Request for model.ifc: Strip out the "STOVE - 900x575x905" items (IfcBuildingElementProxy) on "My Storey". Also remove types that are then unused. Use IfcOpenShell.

First a look at what the model holds.

```python
import ifcopenshell
import ifcopenshell.util.element

model = ifcopenshell.open("model.ifc")
print(model.schema)
storey = next(s for s in model.by_type("IfcBuildingStorey") if s.Name == "My Storey")
proxies = [e for e in ifcopenshell.util.element.get_decomposition(storey) if e.is_a("IfcBuildingElementProxy")]
seen = {}
for e in proxies:
    element_type = ifcopenshell.util.element.get_type(e)
    name = element_type.Name if element_type not in (None, e) else None
    seen[name] = seen.get(name, 0) + 1
for name, count in sorted(seen.items(), key=str):
    print(count, "x", name)
```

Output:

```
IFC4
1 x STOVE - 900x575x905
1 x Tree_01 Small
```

```python
import ifcopenshell
import ifcopenshell.api.root
import ifcopenshell.util.element

model = ifcopenshell.open("model.ifc")

storey = next(s for s in model.by_type("IfcBuildingStorey") if s.Name == "My Storey")
proxies = [e for e in ifcopenshell.util.element.get_decomposition(storey) if e.is_a("IfcBuildingElementProxy")]
targets = [e for e in proxies if (t := ifcopenshell.util.element.get_type(e)) not in (None, e) and t.Name == "STOVE - 900x575x905"]
types = {ifcopenshell.util.element.get_type(e) for e in targets} - {None, *targets}

for e in targets:
    ifcopenshell.api.root.remove_product(model, product=e)
print(len(targets), "removed")

unused = [t for t in types if not ifcopenshell.util.element.get_types(t)]
for t in unused:
    ifcopenshell.api.root.remove_product(model, product=t)
print(len(unused), "unused types removed")

model.write("model-out.ifc")
```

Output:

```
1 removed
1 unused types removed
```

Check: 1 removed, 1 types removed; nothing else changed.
